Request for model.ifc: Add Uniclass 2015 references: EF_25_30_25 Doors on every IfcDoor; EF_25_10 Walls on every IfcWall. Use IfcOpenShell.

First a look at what the model holds.

```python
import ifcopenshell

model = ifcopenshell.open("model.ifc")
print(model.schema)
print("classifications:", [c.Name for c in model.by_type("IfcClassification")])
for ifc_class in ("IfcDoor", "IfcRoof", "IfcStair", "IfcWall", "IfcWindow"):
    print(ifc_class, len(model.by_type(ifc_class)))
```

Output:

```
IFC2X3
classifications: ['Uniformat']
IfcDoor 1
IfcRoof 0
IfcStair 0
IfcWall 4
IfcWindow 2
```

```python
import ifcopenshell
import ifcopenshell.api.classification

model = ifcopenshell.open("model.ifc")

# IFC2X3 requires Source and Edition and has no link from the project to the system.
system = model.create_entity("IfcClassification", Source="NBS", Edition="2015", Name="Uniclass 2015")

codes = {
    "IfcDoor": ("EF_25_30_25", "Doors"),
    "IfcWall": ("EF_25_10", "Walls"),
}
for ifc_class, (code, name) in codes.items():
    products = model.by_type(ifc_class)
    ifcopenshell.api.classification.add_reference(
        model, products=products, classification=system, identification=code, name=name
    )
    print(code, len(products))

model.write("model-out.ifc")
```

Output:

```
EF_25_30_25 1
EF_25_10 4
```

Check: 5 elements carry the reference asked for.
